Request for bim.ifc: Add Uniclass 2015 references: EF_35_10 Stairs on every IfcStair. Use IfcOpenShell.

First a look at what the model holds.

```python
import ifcopenshell

model = ifcopenshell.open("bim.ifc")
print(model.schema)
print("classifications:", [c.Name for c in model.by_type("IfcClassification")])
for ifc_class in ("IfcDoor", "IfcRoof", "IfcStair", "IfcWall", "IfcWindow"):
    print(ifc_class, len(model.by_type(ifc_class)))
```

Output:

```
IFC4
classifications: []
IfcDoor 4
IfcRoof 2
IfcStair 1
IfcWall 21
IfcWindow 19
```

```python
import ifcopenshell
import ifcopenshell.api.classification

model = ifcopenshell.open("bim.ifc")

system = ifcopenshell.api.classification.add_classification(model, classification="Uniclass 2015")

codes = {
    "IfcStair": ("EF_35_10", "Stairs"),
}
for ifc_class, (code, name) in codes.items():
    products = model.by_type(ifc_class)
    ifcopenshell.api.classification.add_reference(
        model, products=products, classification=system, identification=code, name=name
    )
    print(code, len(products))

model.write("bim_v2.ifc")
```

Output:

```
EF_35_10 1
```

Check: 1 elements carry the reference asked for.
